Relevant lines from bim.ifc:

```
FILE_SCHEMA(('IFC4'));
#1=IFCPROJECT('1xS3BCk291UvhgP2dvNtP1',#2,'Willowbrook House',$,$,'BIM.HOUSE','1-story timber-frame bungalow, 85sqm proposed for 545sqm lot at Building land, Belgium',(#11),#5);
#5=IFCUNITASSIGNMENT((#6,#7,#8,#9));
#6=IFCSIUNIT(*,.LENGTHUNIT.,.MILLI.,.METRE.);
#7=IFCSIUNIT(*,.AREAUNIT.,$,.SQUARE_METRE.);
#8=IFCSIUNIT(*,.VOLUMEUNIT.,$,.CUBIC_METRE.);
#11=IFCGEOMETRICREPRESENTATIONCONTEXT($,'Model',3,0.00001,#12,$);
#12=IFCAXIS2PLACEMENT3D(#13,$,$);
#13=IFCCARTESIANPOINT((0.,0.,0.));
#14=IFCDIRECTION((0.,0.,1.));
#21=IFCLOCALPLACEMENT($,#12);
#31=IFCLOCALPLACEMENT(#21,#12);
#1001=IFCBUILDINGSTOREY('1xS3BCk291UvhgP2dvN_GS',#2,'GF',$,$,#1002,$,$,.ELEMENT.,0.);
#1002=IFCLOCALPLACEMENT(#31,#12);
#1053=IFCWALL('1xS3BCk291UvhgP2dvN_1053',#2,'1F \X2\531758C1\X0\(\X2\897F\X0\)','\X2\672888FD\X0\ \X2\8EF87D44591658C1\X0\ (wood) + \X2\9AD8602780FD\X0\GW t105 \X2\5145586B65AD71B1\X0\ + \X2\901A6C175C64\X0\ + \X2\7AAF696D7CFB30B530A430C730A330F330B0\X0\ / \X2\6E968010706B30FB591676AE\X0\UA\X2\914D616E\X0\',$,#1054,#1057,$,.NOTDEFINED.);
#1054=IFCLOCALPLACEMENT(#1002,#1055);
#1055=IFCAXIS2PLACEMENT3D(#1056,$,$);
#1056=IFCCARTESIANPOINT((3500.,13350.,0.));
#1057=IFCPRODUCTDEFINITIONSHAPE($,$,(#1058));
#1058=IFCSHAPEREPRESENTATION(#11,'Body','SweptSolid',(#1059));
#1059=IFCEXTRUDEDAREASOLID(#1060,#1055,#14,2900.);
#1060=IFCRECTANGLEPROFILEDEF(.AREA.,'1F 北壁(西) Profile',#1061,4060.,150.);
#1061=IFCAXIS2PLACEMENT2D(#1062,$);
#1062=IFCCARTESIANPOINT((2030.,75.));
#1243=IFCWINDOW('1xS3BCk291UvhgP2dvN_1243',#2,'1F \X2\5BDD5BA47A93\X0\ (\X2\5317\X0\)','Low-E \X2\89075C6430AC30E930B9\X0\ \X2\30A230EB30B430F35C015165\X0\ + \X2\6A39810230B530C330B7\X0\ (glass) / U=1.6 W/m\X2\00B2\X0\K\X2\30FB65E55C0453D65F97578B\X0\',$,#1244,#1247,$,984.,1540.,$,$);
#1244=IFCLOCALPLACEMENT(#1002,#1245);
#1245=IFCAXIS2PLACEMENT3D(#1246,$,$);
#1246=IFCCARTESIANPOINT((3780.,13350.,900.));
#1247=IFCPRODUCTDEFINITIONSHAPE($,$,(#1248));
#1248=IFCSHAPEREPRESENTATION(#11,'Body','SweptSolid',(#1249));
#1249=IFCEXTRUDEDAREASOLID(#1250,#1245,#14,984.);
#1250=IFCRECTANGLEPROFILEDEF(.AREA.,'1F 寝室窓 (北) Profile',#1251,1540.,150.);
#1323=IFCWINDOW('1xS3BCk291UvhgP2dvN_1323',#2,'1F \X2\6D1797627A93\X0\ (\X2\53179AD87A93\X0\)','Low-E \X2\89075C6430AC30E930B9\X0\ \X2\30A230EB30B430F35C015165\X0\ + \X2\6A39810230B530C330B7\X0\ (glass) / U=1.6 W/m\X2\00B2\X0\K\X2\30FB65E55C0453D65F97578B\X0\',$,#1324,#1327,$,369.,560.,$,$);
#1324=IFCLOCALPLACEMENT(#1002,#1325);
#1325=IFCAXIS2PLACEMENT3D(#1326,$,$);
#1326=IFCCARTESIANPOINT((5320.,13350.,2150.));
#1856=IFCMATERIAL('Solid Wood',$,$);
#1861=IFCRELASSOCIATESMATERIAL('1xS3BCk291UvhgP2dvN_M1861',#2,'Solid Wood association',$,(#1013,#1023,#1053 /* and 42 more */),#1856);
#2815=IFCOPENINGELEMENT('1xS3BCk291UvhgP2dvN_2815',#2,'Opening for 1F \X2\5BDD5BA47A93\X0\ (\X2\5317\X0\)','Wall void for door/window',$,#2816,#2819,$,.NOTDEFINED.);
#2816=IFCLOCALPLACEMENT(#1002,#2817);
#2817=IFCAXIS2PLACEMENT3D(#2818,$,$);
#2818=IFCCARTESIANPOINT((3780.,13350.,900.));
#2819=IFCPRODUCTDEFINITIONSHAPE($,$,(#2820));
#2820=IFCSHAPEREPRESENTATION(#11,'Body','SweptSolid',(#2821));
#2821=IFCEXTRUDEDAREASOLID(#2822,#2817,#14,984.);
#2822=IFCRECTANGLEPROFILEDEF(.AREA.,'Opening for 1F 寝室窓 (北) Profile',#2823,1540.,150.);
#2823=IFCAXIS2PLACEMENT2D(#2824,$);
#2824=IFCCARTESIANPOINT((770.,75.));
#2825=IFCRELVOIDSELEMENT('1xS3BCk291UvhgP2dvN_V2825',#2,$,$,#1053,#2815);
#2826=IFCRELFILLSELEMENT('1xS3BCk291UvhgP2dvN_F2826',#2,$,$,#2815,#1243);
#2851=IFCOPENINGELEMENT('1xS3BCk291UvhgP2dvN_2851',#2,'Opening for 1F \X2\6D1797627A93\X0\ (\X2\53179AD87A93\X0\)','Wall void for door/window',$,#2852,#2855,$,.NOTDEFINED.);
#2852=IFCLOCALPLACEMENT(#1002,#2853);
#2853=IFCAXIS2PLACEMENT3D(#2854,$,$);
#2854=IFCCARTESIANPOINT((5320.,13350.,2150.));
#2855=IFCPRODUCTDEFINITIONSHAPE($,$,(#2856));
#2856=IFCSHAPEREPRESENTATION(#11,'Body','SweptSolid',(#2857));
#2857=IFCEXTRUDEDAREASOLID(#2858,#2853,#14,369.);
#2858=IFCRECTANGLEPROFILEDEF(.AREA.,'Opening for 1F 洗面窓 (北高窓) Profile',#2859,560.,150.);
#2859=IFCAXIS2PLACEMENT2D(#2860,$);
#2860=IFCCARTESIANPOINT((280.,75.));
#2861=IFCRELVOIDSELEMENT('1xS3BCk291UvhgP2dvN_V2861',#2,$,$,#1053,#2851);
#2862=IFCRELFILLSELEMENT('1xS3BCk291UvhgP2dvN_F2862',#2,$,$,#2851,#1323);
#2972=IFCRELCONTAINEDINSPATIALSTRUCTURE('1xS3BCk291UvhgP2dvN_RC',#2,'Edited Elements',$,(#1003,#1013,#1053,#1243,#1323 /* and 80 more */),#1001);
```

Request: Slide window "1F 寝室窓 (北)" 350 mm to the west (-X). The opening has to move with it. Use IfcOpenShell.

```python
import ifcopenshell
import ifcopenshell.api.geometry
import ifcopenshell.util.placement

model = ifcopenshell.open("bim.ifc")

window = model.by_guid("1xS3BCk291UvhgP2dvN_1243")
opening = window.FillsVoids[0].RelatingOpeningElement
wall = opening.VoidsElements[0].RelatingBuildingElement

wall_matrix = ifcopenshell.util.placement.get_local_placement(wall.ObjectPlacement)
shift = wall_matrix[:3, 0] * -350.0
before = ifcopenshell.util.placement.get_local_placement(window.ObjectPlacement)[:3, 3].copy()

# The window is not placed relative to its opening, so move both.
for product in (opening, window):
    matrix = ifcopenshell.util.placement.get_local_placement(product.ObjectPlacement)
    matrix[:3, 3] += shift
    ifcopenshell.api.geometry.edit_object_placement(model, product=product, matrix=matrix, is_si=False)

after = ifcopenshell.util.placement.get_local_placement(window.ObjectPlacement)[:3, 3]
print("window moved by", (after - before).round(3) + 0.0)

model.write("bim_edited.ifc")
```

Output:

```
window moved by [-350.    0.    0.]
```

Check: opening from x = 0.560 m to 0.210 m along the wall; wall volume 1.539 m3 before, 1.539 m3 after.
